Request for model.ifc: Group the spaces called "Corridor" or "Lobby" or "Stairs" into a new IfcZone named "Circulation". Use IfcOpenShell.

First a look at what the model holds.

```python
import ifcopenshell

model = ifcopenshell.open("model.ifc")
print(model.schema)
seen = {}
for space in model.by_type("IfcSpace"):
    seen[space.LongName] = seen.get(space.LongName, 0) + 1
for name, count in sorted(seen.items(), key=str):
    print(count, "x", name)
print("zones:", [z.Name for z in model.by_type("IfcZone")][:20])
```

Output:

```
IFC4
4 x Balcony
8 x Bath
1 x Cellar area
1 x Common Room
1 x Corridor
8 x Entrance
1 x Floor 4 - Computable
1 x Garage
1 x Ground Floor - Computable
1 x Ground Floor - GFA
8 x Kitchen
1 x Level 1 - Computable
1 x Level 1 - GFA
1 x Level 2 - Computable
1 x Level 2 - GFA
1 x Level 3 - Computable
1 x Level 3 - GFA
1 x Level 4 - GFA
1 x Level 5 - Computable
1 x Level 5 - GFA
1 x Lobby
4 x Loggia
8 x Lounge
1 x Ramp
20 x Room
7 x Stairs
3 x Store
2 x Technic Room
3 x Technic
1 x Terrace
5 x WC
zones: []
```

```python
import ifcopenshell
import ifcopenshell.api.group
import ifcopenshell.api.root

model = ifcopenshell.open("model.ifc")

names = {"Corridor", "Lobby", "Stairs"}
spaces = [s for s in model.by_type("IfcSpace") if s.LongName in names]

zone = ifcopenshell.api.root.create_entity(model, ifc_class="IfcZone", name="Circulation")
ifcopenshell.api.group.assign_group(model, products=spaces, group=zone)
print(len(spaces), "spaces in", zone.Name)

model.write("model_updated.ifc")
```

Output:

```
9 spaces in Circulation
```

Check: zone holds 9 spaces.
